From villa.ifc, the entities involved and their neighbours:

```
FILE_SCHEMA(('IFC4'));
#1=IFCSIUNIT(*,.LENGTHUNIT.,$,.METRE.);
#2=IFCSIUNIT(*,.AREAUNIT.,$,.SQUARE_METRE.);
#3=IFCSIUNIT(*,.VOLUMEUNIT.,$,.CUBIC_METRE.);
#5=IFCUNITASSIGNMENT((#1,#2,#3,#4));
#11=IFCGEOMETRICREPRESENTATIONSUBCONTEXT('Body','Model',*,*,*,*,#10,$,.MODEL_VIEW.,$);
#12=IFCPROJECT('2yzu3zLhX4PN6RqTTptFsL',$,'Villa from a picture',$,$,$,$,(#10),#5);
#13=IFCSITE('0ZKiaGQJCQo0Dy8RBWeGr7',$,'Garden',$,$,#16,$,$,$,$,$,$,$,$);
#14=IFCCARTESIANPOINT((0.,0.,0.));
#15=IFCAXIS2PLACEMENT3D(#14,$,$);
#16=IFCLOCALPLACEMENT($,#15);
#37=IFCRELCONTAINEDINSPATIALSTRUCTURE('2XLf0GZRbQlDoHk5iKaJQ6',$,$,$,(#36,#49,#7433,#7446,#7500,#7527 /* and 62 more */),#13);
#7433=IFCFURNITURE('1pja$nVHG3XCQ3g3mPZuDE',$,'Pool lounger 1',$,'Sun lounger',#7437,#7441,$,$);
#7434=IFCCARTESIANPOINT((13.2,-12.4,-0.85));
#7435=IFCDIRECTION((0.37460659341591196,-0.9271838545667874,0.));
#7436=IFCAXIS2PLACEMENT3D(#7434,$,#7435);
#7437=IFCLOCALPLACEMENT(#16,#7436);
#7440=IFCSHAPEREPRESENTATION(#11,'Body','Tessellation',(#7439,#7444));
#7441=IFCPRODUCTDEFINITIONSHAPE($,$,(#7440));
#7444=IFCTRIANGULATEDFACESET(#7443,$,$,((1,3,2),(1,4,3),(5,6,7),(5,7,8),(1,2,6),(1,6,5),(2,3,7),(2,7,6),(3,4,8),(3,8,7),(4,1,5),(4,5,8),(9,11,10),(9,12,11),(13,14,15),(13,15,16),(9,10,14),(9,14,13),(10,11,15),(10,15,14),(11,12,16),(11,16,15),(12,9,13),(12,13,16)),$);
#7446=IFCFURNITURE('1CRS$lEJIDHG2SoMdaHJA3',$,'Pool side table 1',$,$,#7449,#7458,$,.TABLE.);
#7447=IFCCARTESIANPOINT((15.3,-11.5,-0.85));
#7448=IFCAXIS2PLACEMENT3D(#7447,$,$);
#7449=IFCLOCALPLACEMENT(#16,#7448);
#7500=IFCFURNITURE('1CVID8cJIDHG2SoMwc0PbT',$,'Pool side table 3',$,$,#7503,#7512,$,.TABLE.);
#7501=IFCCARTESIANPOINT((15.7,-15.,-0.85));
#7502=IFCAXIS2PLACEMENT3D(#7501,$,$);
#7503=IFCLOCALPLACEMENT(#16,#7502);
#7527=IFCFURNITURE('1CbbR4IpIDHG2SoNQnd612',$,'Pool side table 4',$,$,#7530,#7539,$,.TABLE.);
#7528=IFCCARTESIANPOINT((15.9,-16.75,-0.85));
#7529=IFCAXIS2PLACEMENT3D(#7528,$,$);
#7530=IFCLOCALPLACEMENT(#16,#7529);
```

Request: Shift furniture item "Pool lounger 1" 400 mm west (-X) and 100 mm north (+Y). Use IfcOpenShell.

```python
import ifcopenshell
import ifcopenshell.api.geometry
import ifcopenshell.util.placement

model = ifcopenshell.open("villa.ifc")

item = model.by_guid("1pja$nVHG3XCQ3g3mPZuDE")
matrix = ifcopenshell.util.placement.get_local_placement(item.ObjectPlacement)
matrix[0, 3] -= 0.4
matrix[1, 3] += 0.1
ifcopenshell.api.geometry.edit_object_placement(model, product=item, matrix=matrix, is_si=False)

print(ifcopenshell.util.placement.get_local_placement(item.ObjectPlacement).round(3) + 0.0)

model.write("villa_rev.ifc")
```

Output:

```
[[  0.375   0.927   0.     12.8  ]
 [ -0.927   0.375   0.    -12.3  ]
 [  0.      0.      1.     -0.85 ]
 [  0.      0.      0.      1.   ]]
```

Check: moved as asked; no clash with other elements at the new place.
